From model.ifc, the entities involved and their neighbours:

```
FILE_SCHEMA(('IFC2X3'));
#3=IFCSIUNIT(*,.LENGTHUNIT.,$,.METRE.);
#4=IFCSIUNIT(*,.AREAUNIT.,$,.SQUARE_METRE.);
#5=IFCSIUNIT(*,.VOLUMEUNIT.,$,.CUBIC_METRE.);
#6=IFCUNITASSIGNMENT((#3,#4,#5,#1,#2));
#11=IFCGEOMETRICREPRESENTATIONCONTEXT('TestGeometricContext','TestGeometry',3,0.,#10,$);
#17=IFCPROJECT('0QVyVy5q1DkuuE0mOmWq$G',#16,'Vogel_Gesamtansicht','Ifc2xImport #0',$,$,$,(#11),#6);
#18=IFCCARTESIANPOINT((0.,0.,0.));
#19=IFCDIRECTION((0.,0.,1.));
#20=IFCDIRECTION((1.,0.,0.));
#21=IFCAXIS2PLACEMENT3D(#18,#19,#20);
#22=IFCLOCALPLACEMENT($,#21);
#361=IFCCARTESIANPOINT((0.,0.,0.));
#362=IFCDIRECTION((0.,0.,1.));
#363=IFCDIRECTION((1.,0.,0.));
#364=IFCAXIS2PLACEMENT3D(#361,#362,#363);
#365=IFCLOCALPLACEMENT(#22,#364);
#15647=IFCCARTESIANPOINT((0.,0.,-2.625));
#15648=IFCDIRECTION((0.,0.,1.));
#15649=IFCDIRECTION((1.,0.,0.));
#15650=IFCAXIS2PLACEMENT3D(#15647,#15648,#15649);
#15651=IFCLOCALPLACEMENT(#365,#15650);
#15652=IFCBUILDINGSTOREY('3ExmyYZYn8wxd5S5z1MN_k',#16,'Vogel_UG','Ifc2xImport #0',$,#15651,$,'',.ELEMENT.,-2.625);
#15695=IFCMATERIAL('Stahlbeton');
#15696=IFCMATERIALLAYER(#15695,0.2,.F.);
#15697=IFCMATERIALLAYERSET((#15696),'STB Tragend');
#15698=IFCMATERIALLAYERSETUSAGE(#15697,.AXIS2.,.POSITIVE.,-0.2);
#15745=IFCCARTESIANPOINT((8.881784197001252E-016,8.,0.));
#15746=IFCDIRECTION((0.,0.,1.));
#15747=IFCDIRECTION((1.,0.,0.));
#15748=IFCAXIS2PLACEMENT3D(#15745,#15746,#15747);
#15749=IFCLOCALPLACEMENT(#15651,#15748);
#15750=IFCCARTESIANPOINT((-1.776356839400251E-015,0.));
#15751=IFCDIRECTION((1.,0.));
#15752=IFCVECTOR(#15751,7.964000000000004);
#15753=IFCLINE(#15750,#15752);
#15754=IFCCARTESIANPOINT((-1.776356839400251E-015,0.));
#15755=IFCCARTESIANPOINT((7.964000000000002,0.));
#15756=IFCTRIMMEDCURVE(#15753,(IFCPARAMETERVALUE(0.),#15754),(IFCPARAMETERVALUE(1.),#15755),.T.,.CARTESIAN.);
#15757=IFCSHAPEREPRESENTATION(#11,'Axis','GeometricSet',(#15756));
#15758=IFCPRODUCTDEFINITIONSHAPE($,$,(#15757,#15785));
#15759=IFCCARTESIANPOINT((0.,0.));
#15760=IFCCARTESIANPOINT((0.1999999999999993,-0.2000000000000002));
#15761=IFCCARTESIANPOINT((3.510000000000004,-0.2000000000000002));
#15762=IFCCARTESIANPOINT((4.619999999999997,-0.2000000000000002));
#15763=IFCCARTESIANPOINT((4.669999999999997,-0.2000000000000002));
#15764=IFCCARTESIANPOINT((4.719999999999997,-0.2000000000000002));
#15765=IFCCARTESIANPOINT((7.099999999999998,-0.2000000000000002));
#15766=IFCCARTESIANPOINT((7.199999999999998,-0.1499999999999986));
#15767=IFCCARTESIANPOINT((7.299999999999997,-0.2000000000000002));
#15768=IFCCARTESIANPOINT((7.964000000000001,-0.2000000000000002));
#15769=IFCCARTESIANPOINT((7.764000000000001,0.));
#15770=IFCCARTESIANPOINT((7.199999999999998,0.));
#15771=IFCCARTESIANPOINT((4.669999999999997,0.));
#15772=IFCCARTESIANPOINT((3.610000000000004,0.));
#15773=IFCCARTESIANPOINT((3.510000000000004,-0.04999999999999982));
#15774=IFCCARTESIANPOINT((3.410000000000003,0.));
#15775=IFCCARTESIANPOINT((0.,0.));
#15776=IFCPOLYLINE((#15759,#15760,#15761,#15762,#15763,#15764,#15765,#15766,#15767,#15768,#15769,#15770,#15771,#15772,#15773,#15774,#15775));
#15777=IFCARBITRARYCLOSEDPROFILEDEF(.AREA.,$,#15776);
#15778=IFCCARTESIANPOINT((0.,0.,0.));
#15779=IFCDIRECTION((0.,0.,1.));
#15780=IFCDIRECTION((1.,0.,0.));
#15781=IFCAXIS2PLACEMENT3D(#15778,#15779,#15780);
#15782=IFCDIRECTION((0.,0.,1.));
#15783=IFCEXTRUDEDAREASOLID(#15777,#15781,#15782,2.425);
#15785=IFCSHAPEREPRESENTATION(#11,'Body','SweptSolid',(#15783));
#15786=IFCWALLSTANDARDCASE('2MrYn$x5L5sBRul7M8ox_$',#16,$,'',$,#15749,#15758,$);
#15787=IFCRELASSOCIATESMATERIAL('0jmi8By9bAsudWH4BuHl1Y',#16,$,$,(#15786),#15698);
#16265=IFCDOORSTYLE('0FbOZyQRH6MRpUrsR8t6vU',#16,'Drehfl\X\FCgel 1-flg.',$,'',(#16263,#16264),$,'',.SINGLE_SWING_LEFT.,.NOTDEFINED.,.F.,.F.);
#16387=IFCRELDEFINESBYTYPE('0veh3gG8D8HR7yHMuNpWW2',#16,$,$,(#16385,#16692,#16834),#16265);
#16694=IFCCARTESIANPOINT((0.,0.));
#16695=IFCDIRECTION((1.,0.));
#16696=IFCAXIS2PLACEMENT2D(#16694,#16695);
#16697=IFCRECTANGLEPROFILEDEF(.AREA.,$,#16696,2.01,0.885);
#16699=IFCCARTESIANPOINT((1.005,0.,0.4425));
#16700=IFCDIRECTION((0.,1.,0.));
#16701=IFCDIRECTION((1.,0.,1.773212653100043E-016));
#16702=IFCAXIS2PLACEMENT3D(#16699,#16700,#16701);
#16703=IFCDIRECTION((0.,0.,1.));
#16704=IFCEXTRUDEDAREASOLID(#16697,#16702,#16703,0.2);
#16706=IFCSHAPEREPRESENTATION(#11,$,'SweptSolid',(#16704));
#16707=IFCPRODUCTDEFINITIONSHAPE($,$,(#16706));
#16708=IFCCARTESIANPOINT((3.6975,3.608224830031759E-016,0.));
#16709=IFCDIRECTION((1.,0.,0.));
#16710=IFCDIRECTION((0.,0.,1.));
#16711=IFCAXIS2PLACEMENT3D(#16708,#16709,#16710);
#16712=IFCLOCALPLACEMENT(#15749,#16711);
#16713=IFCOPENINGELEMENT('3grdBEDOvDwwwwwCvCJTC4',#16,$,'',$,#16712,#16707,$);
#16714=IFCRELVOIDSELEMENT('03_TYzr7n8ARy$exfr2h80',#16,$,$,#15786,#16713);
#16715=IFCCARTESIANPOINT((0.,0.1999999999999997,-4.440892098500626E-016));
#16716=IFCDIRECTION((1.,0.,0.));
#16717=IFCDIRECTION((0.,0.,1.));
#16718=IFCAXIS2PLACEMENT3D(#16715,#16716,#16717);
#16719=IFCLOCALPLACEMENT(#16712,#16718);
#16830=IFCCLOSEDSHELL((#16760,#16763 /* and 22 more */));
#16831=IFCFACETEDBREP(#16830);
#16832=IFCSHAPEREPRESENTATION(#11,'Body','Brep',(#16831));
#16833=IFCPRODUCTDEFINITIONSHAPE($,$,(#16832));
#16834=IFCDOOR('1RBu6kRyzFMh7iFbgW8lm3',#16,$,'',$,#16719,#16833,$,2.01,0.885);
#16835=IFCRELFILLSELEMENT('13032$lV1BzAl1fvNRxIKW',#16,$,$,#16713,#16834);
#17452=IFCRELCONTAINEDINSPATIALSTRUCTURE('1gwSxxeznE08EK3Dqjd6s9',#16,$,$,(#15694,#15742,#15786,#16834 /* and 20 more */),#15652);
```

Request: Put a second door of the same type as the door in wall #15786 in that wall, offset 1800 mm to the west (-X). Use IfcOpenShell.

```python
import ifcopenshell
import ifcopenshell.api.feature
import ifcopenshell.api.geometry
import ifcopenshell.api.root
import ifcopenshell.geom
import ifcopenshell.util.element
import ifcopenshell.util.placement
import ifcopenshell.util.shape

model = ifcopenshell.open("model.ifc")
settings = ifcopenshell.geom.settings()


def volume(element):
    """Net volume in cubic metres, openings subtracted."""
    shape = ifcopenshell.geom.create_shape(settings, element)
    return ifcopenshell.util.shape.get_volume(shape.geometry)


door = model.by_guid("1RBu6kRyzFMh7iFbgW8lm3")
opening = door.FillsVoids[0].RelatingOpeningElement
wall = opening.VoidsElements[0].RelatingBuildingElement
before = volume(wall)
shift = ifcopenshell.util.placement.get_local_placement(wall.ObjectPlacement)[:3, 0] * -1.8

# copy_class copies the void relationship, type, container and properties, but no geometry.
new_opening = ifcopenshell.api.root.copy_class(model, product=opening)
new_opening.Representation = ifcopenshell.util.element.copy_deep(
    model, opening.Representation, exclude=["IfcGeometricRepresentationContext", "IfcRepresentationMap"]
)
new_door = ifcopenshell.api.root.copy_class(model, product=door)
new_door.Representation = ifcopenshell.util.element.copy_deep(
    model, door.Representation, exclude=["IfcGeometricRepresentationContext", "IfcRepresentationMap"]
)
fills = ifcopenshell.api.feature.add_filling(model, opening=new_opening, element=new_door)
fills.OwnerHistory = new_door.OwnerHistory  # required in IFC2X3

for old, new in ((opening, new_opening), (door, new_door)):
    matrix = ifcopenshell.util.placement.get_local_placement(old.ObjectPlacement)
    matrix[:3, 3] += shift
    ifcopenshell.api.geometry.edit_object_placement(model, product=new, matrix=matrix, is_si=False)

after = volume(wall)

print(f"wall volume {before:.3f} -> {after:.3f} m3")

model.write("model_edited.ifc")
```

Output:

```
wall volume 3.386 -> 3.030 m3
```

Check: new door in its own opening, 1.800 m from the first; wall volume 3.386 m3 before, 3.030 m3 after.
